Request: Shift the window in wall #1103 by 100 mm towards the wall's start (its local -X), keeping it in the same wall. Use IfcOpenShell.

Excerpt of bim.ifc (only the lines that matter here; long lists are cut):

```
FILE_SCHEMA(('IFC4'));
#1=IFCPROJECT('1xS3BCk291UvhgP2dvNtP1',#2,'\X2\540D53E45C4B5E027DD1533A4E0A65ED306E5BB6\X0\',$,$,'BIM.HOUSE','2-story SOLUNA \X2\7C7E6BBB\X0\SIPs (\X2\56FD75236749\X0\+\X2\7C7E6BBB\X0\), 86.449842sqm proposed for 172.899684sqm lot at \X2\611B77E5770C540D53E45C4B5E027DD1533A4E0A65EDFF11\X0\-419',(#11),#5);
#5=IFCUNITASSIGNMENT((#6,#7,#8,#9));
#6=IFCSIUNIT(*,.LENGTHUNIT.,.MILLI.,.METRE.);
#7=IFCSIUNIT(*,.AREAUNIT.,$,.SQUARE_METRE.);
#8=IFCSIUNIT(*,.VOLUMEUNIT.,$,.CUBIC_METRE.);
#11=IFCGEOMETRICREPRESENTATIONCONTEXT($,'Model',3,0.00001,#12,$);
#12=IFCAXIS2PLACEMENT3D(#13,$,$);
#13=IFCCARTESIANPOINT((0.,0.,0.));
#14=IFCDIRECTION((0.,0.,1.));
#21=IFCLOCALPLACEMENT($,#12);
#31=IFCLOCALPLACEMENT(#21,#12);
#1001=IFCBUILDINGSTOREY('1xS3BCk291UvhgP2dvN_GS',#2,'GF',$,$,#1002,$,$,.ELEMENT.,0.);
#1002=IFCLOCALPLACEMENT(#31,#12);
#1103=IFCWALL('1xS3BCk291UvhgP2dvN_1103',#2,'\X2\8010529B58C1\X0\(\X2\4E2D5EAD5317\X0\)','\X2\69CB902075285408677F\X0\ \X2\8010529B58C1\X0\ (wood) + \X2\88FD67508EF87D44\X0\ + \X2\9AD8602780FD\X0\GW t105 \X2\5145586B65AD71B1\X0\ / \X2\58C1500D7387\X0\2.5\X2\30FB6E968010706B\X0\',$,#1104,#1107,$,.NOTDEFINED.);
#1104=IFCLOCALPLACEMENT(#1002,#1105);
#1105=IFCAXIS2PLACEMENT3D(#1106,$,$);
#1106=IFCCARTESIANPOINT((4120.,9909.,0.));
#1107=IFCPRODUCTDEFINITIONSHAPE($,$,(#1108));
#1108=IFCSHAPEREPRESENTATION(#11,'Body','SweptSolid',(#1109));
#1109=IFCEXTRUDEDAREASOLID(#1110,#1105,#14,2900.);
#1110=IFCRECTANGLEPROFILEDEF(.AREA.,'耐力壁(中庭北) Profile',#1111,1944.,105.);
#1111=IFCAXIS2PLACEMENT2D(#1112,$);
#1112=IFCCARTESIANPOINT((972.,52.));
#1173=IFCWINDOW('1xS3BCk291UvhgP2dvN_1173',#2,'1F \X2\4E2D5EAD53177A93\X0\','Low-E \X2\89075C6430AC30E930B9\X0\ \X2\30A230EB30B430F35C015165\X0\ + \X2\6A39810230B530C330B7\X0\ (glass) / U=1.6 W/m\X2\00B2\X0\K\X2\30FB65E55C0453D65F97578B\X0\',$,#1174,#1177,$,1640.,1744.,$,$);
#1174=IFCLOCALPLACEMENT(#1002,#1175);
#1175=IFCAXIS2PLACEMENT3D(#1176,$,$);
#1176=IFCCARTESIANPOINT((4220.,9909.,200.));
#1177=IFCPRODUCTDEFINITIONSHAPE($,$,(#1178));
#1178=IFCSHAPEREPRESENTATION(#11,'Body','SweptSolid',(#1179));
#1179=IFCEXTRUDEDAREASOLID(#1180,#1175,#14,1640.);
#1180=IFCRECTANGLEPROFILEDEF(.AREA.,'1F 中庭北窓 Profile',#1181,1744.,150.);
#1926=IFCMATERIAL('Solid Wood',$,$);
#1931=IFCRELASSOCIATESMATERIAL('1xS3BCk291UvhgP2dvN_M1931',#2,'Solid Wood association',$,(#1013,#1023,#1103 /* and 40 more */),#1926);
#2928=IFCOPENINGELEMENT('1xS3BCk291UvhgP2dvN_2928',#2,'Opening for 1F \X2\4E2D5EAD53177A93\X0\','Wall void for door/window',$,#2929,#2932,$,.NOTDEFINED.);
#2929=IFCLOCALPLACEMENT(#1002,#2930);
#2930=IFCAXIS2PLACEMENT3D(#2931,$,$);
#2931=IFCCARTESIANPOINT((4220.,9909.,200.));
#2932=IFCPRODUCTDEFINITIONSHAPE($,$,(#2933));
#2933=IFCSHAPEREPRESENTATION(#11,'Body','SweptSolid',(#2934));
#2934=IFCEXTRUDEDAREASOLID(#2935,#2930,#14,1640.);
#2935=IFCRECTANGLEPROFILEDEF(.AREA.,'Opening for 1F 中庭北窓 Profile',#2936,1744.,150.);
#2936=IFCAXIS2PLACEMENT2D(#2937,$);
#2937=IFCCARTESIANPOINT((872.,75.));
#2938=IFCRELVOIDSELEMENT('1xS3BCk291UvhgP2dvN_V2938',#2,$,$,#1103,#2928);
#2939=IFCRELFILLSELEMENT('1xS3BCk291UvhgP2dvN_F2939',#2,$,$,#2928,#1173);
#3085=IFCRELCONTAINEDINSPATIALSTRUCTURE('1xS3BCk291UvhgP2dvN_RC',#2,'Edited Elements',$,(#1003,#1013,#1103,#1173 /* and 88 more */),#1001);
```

```python
import ifcopenshell
import ifcopenshell.api.geometry
import ifcopenshell.util.placement
import ifcopenshell.util.unit

model = ifcopenshell.open("bim.ifc")
unit_scale = ifcopenshell.util.unit.calculate_unit_scale(model)

window = model.by_guid("1xS3BCk291UvhgP2dvN_1173")
opening = window.FillsVoids[0].RelatingOpeningElement
wall = opening.VoidsElements[0].RelatingBuildingElement

wall_matrix = ifcopenshell.util.placement.get_local_placement(wall.ObjectPlacement)
shift = wall_matrix[:3, 0] * -0.1 / unit_scale
before = ifcopenshell.util.placement.get_local_placement(window.ObjectPlacement)[:3, 3].copy()

# The window is not placed relative to its opening, so move both.
for product in (opening, window):
    matrix = ifcopenshell.util.placement.get_local_placement(product.ObjectPlacement)
    matrix[:3, 3] += shift
    ifcopenshell.api.geometry.edit_object_placement(model, product=product, matrix=matrix, is_si=False)

after = ifcopenshell.util.placement.get_local_placement(window.ObjectPlacement)[:3, 3]
print("window moved by", (after - before).round(3) + 0.0)

model.write("bim_edited.ifc")
```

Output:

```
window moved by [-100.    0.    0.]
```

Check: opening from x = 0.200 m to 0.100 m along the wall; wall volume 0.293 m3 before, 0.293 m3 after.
